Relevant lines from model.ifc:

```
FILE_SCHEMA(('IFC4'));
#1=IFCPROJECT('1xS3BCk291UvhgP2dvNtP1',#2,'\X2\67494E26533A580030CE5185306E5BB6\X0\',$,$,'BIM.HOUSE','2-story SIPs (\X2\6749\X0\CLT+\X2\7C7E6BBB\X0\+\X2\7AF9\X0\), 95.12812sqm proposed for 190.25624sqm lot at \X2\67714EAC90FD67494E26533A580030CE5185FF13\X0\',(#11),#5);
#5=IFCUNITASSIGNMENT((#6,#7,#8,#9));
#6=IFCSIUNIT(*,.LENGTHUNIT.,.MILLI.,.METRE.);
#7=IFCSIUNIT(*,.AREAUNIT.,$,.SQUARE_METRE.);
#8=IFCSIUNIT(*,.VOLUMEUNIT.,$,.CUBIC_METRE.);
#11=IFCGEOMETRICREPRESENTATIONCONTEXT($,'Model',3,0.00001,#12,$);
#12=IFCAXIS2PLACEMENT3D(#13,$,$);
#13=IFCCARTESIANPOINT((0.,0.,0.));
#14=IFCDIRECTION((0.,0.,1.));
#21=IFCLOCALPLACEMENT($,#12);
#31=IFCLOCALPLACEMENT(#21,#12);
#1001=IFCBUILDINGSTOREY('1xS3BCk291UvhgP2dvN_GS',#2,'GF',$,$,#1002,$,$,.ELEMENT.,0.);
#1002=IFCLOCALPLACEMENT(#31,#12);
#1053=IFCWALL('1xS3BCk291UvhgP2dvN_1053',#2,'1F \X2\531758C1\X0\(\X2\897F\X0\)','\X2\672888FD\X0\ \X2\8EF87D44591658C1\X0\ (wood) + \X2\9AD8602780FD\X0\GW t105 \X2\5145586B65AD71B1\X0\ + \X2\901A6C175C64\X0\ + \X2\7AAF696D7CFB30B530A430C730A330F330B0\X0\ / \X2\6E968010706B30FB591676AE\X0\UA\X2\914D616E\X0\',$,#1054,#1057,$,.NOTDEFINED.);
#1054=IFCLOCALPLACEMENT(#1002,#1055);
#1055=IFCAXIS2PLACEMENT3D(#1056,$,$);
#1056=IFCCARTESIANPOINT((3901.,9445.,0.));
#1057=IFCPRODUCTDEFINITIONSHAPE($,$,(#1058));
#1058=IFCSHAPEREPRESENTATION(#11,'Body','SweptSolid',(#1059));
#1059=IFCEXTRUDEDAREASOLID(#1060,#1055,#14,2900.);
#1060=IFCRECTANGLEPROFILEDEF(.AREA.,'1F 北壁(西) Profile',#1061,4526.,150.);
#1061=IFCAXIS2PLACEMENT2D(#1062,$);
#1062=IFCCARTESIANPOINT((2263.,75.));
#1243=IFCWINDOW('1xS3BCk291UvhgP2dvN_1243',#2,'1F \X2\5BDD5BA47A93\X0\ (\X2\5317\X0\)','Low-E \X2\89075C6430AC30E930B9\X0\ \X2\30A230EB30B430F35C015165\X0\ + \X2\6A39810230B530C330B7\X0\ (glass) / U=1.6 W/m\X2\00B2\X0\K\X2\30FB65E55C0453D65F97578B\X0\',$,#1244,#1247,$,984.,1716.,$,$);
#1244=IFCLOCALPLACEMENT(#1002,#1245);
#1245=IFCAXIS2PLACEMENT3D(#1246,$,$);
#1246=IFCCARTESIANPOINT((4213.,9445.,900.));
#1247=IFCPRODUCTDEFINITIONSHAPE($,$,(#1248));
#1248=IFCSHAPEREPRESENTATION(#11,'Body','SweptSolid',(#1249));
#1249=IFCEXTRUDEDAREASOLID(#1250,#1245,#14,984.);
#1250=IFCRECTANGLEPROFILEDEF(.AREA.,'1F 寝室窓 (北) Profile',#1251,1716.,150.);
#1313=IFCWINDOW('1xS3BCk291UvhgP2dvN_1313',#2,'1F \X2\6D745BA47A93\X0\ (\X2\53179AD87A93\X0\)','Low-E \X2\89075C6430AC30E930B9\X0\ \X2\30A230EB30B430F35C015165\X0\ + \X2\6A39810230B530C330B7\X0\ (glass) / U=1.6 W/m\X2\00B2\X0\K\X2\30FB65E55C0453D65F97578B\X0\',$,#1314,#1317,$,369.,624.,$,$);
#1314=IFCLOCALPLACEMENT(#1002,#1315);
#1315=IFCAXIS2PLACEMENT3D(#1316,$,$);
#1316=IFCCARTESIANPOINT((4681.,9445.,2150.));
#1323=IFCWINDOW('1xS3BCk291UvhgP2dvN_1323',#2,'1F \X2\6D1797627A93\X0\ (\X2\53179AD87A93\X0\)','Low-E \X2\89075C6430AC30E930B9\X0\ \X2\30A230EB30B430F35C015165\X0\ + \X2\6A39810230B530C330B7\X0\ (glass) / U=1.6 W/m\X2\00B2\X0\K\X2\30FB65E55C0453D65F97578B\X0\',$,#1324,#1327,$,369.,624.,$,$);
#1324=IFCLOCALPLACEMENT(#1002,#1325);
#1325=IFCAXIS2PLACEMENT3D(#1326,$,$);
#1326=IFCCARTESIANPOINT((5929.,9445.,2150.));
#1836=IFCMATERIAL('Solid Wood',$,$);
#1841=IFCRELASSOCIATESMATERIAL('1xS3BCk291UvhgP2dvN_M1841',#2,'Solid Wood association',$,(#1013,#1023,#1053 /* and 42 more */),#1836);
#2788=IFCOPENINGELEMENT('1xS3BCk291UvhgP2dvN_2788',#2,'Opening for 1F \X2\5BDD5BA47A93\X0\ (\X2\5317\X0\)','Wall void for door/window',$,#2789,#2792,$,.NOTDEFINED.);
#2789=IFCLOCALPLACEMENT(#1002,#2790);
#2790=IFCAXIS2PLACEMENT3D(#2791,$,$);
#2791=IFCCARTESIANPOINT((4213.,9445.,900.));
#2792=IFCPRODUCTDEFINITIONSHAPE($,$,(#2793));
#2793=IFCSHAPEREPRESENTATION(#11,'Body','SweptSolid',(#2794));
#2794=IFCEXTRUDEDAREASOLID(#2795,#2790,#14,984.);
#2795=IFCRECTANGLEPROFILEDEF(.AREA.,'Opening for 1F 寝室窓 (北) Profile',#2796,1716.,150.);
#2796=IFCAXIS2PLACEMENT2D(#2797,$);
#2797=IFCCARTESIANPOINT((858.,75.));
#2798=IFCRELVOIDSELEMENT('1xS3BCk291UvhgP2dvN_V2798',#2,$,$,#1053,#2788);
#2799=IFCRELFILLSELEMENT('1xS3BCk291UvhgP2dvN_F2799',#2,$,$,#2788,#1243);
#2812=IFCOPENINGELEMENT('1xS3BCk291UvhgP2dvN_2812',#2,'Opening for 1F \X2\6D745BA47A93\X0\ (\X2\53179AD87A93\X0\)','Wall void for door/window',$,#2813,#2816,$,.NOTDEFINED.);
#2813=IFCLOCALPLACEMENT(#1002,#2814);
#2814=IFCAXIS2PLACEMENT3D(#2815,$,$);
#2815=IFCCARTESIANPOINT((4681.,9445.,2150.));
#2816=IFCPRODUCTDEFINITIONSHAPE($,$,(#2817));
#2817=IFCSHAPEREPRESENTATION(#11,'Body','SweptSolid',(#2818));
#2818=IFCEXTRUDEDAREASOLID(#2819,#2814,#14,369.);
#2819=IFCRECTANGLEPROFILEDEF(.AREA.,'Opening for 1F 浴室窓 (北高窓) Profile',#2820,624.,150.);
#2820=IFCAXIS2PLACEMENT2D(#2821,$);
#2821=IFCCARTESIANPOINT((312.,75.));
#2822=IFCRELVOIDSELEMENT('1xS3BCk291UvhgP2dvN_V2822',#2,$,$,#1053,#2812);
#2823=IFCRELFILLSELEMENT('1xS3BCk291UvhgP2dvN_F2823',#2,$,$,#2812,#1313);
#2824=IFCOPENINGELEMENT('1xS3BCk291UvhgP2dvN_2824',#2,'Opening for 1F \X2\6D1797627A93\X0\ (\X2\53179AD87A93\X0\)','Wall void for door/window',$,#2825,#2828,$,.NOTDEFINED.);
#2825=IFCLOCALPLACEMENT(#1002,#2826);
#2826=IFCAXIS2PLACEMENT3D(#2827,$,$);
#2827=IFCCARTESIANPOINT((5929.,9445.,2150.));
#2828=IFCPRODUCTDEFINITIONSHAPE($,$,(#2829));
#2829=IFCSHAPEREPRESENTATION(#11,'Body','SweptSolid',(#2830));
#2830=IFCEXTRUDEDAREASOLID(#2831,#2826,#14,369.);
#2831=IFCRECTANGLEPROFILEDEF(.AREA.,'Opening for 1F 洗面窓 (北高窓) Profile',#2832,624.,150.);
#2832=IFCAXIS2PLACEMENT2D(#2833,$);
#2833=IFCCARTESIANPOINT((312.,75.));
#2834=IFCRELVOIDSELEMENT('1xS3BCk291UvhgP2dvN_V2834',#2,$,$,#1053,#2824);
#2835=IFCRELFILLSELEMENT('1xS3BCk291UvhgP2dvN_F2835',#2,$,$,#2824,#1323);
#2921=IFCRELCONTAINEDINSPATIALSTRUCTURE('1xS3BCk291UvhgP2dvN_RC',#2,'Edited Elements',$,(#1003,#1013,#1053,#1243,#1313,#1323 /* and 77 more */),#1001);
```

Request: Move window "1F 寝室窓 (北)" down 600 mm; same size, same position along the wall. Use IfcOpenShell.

```python
import numpy as np
import ifcopenshell
import ifcopenshell.api.geometry
import ifcopenshell.util.placement
import ifcopenshell.util.unit

model = ifcopenshell.open("model.ifc")
unit_scale = ifcopenshell.util.unit.calculate_unit_scale(model)

window = model.by_id(1243)
opening = window.FillsVoids[0].RelatingOpeningElement
dz = -0.6 / unit_scale

shift = np.array([0.0, 0.0, dz])
# The window is not placed relative to its opening, so move both.
for product in (opening, window):
    matrix = ifcopenshell.util.placement.get_local_placement(product.ObjectPlacement)
    matrix[:3, 3] += shift
    ifcopenshell.api.geometry.edit_object_placement(model, product=product, matrix=matrix, is_si=False)

print(f"moved by {dz * unit_scale:+.3f} m")

model.write("model_rev.ifc")
```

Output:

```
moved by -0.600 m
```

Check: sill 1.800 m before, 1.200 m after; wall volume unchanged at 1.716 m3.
